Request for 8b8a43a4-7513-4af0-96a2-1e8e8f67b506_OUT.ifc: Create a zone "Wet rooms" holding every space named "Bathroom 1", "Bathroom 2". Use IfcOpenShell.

First a look at what the model holds.

```python
import ifcopenshell

model = ifcopenshell.open("8b8a43a4-7513-4af0-96a2-1e8e8f67b506_OUT.ifc")
print(model.schema)
seen = {}
for space in model.by_type("IfcSpace"):
    seen[space.LongName] = seen.get(space.LongName, 0) + 1
for name, count in sorted(seen.items(), key=str):
    print(count, "x", name)
print("zones:", [z.Name for z in model.by_type("IfcZone")][:20])
```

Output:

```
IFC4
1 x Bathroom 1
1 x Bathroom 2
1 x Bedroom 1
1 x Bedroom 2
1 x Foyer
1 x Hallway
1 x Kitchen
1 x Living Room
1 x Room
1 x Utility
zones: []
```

```python
import ifcopenshell
import ifcopenshell.api.group
import ifcopenshell.api.root

model = ifcopenshell.open("8b8a43a4-7513-4af0-96a2-1e8e8f67b506_OUT.ifc")

names = {"Bathroom 1", "Bathroom 2"}
spaces = [s for s in model.by_type("IfcSpace") if s.LongName in names]

zone = ifcopenshell.api.root.create_entity(model, ifc_class="IfcZone", name="Wet rooms")
ifcopenshell.api.group.assign_group(model, products=spaces, group=zone)
print(len(spaces), "spaces in", zone.Name)

model.write("8b8a43a4-7513-4af0-96a2-1e8e8f67b506_OUT_edited.ifc")
```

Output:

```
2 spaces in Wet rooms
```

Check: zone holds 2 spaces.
